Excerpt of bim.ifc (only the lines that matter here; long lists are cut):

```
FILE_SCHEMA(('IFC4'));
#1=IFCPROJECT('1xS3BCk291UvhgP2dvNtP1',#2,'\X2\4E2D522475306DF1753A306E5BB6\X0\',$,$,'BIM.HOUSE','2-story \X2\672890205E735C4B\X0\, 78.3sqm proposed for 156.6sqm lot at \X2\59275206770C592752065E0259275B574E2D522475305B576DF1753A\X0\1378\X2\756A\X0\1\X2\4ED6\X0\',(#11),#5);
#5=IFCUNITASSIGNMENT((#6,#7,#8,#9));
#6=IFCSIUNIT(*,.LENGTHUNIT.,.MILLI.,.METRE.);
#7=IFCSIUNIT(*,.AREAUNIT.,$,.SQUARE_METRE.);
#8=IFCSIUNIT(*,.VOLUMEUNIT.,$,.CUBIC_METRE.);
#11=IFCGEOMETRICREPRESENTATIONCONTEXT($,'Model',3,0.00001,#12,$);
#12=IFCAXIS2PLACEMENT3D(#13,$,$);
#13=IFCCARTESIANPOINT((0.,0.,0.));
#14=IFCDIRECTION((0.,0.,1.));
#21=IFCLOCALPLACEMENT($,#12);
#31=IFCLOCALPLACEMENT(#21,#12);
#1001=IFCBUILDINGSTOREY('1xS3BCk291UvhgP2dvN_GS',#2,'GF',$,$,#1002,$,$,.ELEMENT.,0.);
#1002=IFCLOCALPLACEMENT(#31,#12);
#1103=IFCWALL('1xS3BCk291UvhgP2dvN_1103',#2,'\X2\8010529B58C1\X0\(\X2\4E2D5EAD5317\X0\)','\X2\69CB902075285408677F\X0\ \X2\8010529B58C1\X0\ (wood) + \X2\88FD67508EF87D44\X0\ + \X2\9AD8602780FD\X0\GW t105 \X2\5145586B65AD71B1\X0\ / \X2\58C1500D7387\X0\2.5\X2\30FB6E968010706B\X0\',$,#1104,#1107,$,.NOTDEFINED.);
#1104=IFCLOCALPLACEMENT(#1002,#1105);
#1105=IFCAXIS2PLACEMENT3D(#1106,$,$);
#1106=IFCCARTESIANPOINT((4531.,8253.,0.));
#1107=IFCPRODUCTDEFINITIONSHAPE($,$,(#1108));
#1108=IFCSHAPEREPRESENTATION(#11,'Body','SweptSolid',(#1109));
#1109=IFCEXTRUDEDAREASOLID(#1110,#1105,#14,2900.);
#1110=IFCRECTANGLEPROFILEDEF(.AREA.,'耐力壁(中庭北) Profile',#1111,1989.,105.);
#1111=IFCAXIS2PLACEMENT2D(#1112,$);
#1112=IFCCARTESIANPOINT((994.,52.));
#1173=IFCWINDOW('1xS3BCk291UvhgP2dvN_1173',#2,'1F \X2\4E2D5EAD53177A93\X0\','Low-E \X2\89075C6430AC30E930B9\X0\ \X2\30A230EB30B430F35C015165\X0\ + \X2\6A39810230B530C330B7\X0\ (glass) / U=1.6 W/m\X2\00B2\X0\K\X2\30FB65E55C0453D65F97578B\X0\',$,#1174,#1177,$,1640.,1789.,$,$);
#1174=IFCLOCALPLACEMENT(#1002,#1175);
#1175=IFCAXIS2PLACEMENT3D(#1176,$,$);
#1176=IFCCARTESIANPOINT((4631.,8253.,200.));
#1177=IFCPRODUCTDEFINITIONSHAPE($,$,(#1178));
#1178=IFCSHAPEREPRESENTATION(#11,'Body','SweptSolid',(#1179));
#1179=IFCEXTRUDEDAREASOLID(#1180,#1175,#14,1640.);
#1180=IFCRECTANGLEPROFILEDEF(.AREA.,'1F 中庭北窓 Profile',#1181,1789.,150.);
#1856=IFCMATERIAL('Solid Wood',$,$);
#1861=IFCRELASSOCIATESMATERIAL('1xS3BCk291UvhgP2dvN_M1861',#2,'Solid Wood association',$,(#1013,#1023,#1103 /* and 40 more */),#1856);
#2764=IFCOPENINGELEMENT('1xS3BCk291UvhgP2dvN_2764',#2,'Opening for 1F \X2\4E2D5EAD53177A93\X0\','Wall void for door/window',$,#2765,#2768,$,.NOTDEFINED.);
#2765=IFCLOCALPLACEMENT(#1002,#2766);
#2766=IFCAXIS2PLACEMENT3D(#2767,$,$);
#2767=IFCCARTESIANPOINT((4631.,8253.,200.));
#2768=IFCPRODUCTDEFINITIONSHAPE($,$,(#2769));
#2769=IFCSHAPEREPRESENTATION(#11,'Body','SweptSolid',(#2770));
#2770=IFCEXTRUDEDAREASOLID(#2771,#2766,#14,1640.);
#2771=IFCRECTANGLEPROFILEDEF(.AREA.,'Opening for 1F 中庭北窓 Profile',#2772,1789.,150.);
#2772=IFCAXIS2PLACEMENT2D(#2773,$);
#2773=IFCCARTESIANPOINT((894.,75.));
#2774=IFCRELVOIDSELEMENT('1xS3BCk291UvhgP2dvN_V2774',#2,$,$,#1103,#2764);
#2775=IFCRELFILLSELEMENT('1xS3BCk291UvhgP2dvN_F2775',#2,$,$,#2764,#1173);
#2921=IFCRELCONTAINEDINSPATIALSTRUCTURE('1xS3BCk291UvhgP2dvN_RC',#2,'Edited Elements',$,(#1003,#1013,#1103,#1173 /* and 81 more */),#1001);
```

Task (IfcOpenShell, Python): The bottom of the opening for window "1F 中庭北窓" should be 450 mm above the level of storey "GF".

```python
import numpy as np
import ifcopenshell
import ifcopenshell.api.geometry
import ifcopenshell.geom
import ifcopenshell.util.element
import ifcopenshell.util.placement
import ifcopenshell.util.shape
import ifcopenshell.util.unit

model = ifcopenshell.open("bim.ifc")
unit_scale = ifcopenshell.util.unit.calculate_unit_scale(model)

window = model.by_guid("1xS3BCk291UvhgP2dvN_1173")
opening = window.FillsVoids[0].RelatingOpeningElement
storey = ifcopenshell.util.element.get_container(window, ifc_class="IfcBuildingStorey")
level = ifcopenshell.util.placement.get_local_placement(storey.ObjectPlacement)[2, 3]

# The opening's origin need not be at the sill, so measure its lowest point.
shape = ifcopenshell.geom.create_shape(ifcopenshell.geom.settings(), opening)
bottom = ifcopenshell.util.shape.get_shape_bottom_elevation(shape, shape.geometry) / unit_scale
dz = level + 450.0 - bottom

shift = np.array([0.0, 0.0, dz])
# The window is not placed relative to its opening, so move both.
for product in (opening, window):
    matrix = ifcopenshell.util.placement.get_local_placement(product.ObjectPlacement)
    matrix[:3, 3] += shift
    ifcopenshell.api.geometry.edit_object_placement(model, product=product, matrix=matrix, is_si=False)

print(f"moved by {dz * unit_scale:+.3f} m")

model.write("bim_v2.ifc")
```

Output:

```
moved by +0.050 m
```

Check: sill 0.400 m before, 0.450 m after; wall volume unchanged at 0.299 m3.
